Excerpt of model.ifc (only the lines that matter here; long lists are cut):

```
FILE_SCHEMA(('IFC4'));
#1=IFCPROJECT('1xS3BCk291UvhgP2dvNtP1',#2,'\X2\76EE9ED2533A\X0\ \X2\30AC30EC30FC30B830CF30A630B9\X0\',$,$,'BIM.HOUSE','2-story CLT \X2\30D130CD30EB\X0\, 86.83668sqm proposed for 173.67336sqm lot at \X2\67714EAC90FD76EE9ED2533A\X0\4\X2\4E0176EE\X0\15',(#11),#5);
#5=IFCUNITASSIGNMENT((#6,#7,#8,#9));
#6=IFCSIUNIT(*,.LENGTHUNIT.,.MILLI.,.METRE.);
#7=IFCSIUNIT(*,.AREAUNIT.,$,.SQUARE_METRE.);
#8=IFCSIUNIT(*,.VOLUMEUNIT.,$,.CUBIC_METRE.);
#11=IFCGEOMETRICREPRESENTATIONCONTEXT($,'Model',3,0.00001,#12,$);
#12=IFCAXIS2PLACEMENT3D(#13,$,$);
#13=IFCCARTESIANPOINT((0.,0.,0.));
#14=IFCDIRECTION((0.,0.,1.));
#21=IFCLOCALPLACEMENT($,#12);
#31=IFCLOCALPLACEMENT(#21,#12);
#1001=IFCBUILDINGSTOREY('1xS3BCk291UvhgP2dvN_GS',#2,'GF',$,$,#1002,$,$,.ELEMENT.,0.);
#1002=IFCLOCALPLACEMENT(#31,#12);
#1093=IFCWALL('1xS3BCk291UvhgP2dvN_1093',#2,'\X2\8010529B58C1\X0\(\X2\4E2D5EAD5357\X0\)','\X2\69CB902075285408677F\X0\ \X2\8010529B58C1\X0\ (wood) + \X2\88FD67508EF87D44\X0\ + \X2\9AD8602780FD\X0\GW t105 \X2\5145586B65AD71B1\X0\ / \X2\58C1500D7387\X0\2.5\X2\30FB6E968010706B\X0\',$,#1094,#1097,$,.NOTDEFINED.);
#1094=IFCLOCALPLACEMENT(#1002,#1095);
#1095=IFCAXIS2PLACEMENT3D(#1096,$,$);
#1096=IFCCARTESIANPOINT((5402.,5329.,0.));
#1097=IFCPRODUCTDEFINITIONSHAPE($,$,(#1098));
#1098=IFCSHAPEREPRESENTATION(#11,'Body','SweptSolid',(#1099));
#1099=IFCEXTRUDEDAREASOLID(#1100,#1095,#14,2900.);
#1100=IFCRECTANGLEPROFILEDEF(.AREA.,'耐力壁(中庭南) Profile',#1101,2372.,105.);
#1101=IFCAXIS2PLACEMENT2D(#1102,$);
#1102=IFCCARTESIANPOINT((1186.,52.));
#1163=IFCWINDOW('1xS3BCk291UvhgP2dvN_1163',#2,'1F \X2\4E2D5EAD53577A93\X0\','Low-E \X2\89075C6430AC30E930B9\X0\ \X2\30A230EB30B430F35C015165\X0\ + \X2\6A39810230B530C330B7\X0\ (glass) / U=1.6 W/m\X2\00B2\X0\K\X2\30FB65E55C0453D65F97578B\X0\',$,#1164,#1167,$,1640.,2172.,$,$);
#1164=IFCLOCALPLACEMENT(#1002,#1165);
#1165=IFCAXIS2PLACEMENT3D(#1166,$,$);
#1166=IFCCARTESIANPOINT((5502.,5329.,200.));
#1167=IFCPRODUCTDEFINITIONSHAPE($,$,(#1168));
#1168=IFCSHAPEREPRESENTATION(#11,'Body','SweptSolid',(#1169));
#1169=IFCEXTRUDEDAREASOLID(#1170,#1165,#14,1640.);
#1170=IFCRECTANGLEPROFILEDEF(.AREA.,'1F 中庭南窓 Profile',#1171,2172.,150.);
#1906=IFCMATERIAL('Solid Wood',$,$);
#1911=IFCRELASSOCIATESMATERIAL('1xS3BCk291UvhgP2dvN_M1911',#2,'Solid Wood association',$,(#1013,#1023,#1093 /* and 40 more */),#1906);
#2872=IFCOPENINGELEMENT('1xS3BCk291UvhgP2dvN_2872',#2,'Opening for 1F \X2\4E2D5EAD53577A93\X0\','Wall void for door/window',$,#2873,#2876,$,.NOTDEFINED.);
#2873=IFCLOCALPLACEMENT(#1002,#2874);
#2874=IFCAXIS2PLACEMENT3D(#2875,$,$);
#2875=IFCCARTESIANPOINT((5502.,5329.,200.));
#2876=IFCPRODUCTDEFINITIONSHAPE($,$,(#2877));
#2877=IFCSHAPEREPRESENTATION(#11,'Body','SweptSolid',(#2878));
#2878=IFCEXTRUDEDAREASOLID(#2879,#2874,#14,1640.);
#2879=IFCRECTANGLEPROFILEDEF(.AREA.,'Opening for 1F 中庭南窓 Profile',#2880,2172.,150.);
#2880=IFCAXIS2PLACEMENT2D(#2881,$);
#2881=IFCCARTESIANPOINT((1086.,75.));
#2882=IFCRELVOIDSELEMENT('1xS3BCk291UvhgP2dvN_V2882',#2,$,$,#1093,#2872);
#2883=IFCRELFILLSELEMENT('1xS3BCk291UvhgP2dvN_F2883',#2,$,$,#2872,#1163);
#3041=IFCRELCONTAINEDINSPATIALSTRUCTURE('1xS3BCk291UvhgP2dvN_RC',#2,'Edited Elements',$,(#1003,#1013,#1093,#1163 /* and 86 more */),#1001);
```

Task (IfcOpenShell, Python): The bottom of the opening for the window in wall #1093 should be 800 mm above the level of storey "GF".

```python
import numpy as np
import ifcopenshell
import ifcopenshell.api.geometry
import ifcopenshell.geom
import ifcopenshell.util.element
import ifcopenshell.util.placement
import ifcopenshell.util.shape
import ifcopenshell.util.unit

model = ifcopenshell.open("model.ifc")
unit_scale = ifcopenshell.util.unit.calculate_unit_scale(model)

window = model.by_guid("1xS3BCk291UvhgP2dvN_1163")
opening = window.FillsVoids[0].RelatingOpeningElement
storey = ifcopenshell.util.element.get_container(window, ifc_class="IfcBuildingStorey")
level = ifcopenshell.util.placement.get_local_placement(storey.ObjectPlacement)[2, 3]

# The opening's origin need not be at the sill, so measure its lowest point.
shape = ifcopenshell.geom.create_shape(ifcopenshell.geom.settings(), opening)
bottom = ifcopenshell.util.shape.get_shape_bottom_elevation(shape, shape.geometry) / unit_scale
dz = level + 0.8 / unit_scale - bottom

shift = np.array([0.0, 0.0, dz])
# The window is not placed relative to its opening, so move both.
for product in (opening, window):
    matrix = ifcopenshell.util.placement.get_local_placement(product.ObjectPlacement)
    matrix[:3, 3] += shift
    ifcopenshell.api.geometry.edit_object_placement(model, product=product, matrix=matrix, is_si=False)

print(f"moved by {dz * unit_scale:+.3f} m")

model.write("model_rev.ifc")
```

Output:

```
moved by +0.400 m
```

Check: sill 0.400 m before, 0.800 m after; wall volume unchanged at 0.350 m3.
